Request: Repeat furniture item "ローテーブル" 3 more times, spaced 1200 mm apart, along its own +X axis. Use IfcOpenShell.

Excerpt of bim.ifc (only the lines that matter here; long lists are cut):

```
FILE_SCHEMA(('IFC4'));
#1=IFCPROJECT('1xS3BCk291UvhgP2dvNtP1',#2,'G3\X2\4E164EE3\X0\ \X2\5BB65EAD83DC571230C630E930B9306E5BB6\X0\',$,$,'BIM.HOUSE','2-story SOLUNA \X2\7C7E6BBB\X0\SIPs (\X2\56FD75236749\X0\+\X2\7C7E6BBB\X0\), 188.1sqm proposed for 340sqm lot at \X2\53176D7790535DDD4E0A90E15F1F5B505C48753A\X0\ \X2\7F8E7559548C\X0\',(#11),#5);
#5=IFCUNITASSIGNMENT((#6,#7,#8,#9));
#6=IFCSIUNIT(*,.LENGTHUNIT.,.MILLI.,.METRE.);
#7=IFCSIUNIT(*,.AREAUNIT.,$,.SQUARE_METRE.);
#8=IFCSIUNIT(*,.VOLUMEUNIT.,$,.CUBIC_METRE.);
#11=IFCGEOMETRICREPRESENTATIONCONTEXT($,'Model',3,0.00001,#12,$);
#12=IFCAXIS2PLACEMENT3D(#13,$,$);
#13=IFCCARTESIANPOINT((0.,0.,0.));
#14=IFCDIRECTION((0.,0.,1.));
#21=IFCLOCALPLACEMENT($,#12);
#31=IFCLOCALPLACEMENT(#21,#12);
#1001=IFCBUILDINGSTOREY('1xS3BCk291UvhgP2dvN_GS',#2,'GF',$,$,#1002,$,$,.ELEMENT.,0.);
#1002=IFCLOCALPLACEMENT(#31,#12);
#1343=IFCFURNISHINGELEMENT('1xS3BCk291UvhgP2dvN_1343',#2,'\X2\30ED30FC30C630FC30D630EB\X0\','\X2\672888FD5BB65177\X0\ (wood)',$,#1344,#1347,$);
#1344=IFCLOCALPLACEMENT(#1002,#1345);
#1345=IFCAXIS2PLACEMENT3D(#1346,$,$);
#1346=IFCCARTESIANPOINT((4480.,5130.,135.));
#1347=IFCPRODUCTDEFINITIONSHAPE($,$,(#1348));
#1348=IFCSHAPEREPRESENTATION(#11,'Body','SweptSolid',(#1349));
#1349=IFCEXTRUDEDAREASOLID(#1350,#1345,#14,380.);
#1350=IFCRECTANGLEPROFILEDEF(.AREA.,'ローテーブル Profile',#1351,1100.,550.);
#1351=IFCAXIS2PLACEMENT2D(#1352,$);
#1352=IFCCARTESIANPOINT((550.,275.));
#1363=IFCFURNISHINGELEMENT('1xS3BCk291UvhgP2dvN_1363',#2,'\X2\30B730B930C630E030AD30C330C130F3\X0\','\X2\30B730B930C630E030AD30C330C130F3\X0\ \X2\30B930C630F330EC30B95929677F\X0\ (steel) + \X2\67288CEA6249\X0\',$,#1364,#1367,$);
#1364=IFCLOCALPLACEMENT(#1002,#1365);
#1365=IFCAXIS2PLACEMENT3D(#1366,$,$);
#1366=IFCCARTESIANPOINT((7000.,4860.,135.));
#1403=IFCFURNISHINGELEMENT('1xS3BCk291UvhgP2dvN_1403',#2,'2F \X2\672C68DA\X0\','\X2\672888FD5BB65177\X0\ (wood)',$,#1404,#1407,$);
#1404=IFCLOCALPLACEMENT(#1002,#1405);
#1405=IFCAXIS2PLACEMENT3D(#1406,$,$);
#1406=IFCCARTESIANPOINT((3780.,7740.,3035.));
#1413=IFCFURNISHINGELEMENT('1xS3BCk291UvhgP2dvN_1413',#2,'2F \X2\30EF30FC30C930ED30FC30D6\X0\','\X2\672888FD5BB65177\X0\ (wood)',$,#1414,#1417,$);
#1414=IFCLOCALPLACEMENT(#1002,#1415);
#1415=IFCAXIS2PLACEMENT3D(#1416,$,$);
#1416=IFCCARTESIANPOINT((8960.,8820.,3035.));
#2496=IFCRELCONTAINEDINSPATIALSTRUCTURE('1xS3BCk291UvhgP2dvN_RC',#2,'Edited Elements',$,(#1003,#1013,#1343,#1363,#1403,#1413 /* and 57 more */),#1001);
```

```python
import ifcopenshell
import ifcopenshell.api.geometry
import ifcopenshell.api.root
import ifcopenshell.util.element
import ifcopenshell.util.placement
import ifcopenshell.util.unit

model = ifcopenshell.open("bim.ifc")
unit_scale = ifcopenshell.util.unit.calculate_unit_scale(model)


def reuse_history(source, copy):
    """copy_class also copies each property set's owner history, people and application; keep the originals."""
    for rel in copy.IsDefinedBy:
        if rel.is_a("IfcRelDefinesByProperties") and (history := rel.RelatingPropertyDefinition.OwnerHistory):
            rel.RelatingPropertyDefinition.OwnerHistory = source.OwnerHistory
            ifcopenshell.util.element.remove_deep2(model, history)


source = model.by_id(1343)
base = ifcopenshell.util.placement.get_local_placement(source.ObjectPlacement)
step = base[:3, 0] * 1.2 / unit_scale

for i in range(1, 4):
    copy = ifcopenshell.api.root.copy_class(model, product=source)
    copy.Representation = ifcopenshell.util.element.copy_deep(
        model, source.Representation, exclude=["IfcGeometricRepresentationContext", "IfcRepresentationMap"]
    )
    reuse_history(source, copy)
    matrix = base.copy()
    matrix[:3, 3] += i * step
    print("added at", matrix[:3, 3].round(3) + 0.0)
    ifcopenshell.api.geometry.edit_object_placement(model, product=copy, matrix=matrix, is_si=False)

model.write("bim_updated.ifc")
```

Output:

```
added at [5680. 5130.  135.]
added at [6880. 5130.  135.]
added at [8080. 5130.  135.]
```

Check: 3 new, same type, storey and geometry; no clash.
